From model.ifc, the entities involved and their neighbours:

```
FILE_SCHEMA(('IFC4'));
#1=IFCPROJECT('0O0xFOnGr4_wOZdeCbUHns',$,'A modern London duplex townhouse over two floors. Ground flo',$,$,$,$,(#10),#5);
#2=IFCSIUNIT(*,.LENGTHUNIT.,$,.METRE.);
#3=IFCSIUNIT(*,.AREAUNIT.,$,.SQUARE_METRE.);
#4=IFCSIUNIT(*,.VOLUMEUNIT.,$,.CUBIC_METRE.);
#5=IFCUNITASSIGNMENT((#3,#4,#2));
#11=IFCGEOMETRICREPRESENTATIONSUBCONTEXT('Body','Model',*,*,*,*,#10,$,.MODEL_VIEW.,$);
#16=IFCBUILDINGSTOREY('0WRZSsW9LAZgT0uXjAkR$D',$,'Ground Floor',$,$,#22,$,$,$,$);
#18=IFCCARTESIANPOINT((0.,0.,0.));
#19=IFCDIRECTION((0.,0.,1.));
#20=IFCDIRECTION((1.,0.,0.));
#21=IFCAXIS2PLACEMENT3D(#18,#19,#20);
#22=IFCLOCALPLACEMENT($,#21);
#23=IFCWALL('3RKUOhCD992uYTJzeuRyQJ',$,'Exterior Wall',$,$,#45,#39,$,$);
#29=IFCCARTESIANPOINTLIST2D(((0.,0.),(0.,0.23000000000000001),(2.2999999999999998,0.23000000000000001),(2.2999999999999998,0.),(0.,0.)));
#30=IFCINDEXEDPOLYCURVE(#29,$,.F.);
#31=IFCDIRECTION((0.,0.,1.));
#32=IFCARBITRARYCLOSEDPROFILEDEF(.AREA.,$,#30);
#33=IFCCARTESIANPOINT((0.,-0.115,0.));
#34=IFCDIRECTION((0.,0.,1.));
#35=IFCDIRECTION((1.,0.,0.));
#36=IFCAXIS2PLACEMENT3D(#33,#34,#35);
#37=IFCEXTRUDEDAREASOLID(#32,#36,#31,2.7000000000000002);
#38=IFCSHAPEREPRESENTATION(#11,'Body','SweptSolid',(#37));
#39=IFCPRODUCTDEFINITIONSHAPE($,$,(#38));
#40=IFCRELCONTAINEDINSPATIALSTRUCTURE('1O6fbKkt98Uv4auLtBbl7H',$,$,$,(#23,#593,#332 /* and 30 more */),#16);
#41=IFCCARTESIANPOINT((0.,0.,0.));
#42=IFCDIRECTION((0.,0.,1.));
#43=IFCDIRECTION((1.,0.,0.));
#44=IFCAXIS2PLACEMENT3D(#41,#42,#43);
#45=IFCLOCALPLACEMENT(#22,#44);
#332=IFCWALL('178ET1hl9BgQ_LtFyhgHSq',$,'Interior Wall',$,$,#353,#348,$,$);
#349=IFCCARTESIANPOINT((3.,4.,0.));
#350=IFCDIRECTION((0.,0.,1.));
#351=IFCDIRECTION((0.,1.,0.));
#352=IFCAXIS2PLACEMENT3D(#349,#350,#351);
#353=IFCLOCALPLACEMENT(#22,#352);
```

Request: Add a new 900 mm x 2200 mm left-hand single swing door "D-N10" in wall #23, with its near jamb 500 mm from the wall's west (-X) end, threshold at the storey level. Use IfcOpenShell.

```python
import numpy as np
import ifcopenshell
import ifcopenshell.api.feature
import ifcopenshell.api.geometry
import ifcopenshell.api.root
import ifcopenshell.api.spatial
import ifcopenshell.geom
import ifcopenshell.util.element
import ifcopenshell.util.placement
import ifcopenshell.util.representation
import ifcopenshell.util.shape
import ifcopenshell.util.unit

model = ifcopenshell.open("model.ifc")
unit_scale = ifcopenshell.util.unit.calculate_unit_scale(model)
settings = ifcopenshell.geom.settings()


def volume(element):
    """Net volume in cubic metres, openings subtracted."""
    shape = ifcopenshell.geom.create_shape(settings, element)
    return ifcopenshell.util.shape.get_volume(shape.geometry)


wall = model.by_guid("3RKUOhCD992uYTJzeuRyQJ")
storey = ifcopenshell.util.element.get_container(wall, ifc_class="IfcBuildingStorey")
context = ifcopenshell.util.representation.get_context(model, "Model", "Body", "MODEL_VIEW")
before = volume(wall)

width, height, from_end, sill = 0.9, 2.2, 0.5, 0.0  # metres

# The wall runs along its own X axis, and the end named is its -X end.
wall_shape = ifcopenshell.geom.create_shape(settings, wall)
x, y, z = ifcopenshell.util.shape.get_vertices(wall_shape.geometry).T
start = x.min() + from_end
face, thickness = float(y.min()), float(y.max() - y.min())
wall_matrix = ifcopenshell.util.placement.get_local_placement(wall.ObjectPlacement)
level = ifcopenshell.util.placement.get_local_placement(storey.ObjectPlacement)[2, 3]


def in_wall(x, y):
    """Placement at x, y metres in the wall's axes, at sill height."""
    matrix = wall_matrix.copy()
    matrix[:, 3] = wall_matrix @ np.array([x / unit_scale, y / unit_scale, 0.0, 1.0])
    matrix[2, 3] = level + sill / unit_scale
    return matrix


# Opening: a box that overshoots both wall faces by 50 mm.
opening = ifcopenshell.api.root.create_entity(model, ifc_class="IfcOpeningElement", predefined_type="OPENING")
box = ifcopenshell.api.geometry.add_wall_representation(
    model, context=context, length=width, height=height, thickness=thickness + 0.1
)
ifcopenshell.api.geometry.assign_representation(model, product=opening, representation=box)
ifcopenshell.api.geometry.edit_object_placement(model, product=opening, matrix=in_wall(start, face - 0.05), is_si=False)
ifcopenshell.api.feature.add_feature(model, feature=opening, element=wall)

door = ifcopenshell.api.root.create_entity(model, ifc_class="IfcDoor", name="D-N10", predefined_type="DOOR")
door.OverallWidth, door.OverallHeight = width / unit_scale, height / unit_scale
door.OperationType = "SINGLE_SWING_LEFT"
body = ifcopenshell.api.geometry.add_door_representation(
    model,
    context=context,
    overall_width=door.OverallWidth,
    overall_height=door.OverallHeight,
    operation_type="SINGLE_SWING_LEFT",
    lining_properties={"LiningDepth": thickness / unit_scale, "ThresholdDepth": thickness / unit_scale},
)
ifcopenshell.api.geometry.assign_representation(model, product=door, representation=body)
ifcopenshell.api.spatial.assign_container(model, products=[door], relating_structure=storey)
ifcopenshell.api.feature.add_filling(model, opening=opening, element=door)

# The lining spans the wall, so the door starts at the wall face.
ifcopenshell.api.geometry.edit_object_placement(model, product=door, matrix=in_wall(start, face), is_si=False)

after = volume(wall)

print(f"wall volume {before:.3f} -> {after:.3f} m3")

model.write("model_v2.ifc")
```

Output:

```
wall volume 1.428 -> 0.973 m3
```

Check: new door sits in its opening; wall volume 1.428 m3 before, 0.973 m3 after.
